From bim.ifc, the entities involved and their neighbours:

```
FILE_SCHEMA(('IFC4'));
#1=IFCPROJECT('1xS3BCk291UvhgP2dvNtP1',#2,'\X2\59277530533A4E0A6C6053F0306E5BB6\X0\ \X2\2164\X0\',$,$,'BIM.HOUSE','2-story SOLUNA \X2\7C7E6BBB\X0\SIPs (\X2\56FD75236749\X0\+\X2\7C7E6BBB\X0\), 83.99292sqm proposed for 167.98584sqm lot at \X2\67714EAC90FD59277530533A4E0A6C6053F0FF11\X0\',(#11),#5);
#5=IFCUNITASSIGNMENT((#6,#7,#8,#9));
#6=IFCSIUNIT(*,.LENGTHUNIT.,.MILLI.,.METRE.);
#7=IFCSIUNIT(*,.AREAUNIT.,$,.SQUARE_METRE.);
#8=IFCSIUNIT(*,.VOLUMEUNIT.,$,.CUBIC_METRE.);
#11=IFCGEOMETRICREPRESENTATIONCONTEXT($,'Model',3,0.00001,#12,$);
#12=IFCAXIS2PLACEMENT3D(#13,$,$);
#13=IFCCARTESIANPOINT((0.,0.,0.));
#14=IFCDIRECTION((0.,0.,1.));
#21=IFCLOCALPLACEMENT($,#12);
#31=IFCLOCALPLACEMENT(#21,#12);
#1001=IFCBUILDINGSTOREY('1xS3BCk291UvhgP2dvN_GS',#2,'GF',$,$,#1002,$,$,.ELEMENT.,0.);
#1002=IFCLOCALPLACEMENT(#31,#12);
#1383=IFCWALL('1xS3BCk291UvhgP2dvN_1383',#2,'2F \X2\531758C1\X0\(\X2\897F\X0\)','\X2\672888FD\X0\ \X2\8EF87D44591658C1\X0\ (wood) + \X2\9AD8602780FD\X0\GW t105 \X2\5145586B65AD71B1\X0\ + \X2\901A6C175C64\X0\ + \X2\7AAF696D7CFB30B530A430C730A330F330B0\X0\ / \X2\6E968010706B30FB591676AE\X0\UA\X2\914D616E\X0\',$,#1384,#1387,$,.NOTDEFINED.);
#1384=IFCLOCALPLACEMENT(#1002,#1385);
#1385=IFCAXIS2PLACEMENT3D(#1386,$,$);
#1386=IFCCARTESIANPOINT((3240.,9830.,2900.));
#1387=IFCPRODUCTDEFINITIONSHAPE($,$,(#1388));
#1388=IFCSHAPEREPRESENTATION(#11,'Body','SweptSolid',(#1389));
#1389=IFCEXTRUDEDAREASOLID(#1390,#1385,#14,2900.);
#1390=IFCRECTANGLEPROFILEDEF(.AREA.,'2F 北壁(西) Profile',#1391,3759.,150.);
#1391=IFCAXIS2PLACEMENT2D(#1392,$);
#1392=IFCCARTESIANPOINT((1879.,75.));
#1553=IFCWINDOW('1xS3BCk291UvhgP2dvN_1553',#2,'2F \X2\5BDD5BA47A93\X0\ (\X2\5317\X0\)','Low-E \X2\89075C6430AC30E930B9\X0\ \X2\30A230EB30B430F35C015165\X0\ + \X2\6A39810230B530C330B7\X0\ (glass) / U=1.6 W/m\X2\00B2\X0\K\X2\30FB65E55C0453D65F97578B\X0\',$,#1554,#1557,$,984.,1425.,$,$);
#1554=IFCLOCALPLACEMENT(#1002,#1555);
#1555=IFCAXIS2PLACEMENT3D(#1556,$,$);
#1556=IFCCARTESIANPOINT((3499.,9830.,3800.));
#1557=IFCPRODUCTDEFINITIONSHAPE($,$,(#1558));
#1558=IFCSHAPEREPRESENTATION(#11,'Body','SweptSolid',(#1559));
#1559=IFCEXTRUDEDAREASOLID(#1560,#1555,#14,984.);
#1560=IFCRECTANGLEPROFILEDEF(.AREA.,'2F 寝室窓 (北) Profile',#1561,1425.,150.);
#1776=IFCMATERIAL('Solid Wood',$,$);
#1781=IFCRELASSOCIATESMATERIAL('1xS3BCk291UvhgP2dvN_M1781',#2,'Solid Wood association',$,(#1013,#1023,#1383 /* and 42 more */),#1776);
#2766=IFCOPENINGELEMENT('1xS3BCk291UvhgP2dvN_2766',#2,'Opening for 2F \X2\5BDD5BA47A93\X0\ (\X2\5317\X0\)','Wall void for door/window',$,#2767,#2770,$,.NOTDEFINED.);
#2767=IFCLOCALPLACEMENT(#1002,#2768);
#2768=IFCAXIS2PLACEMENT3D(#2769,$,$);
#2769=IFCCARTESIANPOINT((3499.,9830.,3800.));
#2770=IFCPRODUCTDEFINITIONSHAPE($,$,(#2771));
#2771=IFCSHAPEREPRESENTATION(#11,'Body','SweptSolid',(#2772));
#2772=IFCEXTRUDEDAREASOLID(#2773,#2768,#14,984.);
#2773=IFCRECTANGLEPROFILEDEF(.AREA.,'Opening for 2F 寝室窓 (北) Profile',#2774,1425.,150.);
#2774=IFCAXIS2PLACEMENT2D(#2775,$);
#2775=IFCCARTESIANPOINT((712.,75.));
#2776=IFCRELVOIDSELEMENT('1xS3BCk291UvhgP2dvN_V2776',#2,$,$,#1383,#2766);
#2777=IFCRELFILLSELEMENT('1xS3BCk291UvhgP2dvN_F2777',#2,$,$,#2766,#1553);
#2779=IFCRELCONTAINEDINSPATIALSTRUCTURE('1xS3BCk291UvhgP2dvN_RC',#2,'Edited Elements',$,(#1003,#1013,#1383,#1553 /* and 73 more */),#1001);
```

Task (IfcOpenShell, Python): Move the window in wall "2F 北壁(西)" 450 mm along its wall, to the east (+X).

```python
import ifcopenshell
import ifcopenshell.api.geometry
import ifcopenshell.util.placement
import ifcopenshell.util.unit

model = ifcopenshell.open("bim.ifc")
unit_scale = ifcopenshell.util.unit.calculate_unit_scale(model)

window = model.by_guid("1xS3BCk291UvhgP2dvN_1553")
opening = window.FillsVoids[0].RelatingOpeningElement
wall = opening.VoidsElements[0].RelatingBuildingElement

wall_matrix = ifcopenshell.util.placement.get_local_placement(wall.ObjectPlacement)
shift = wall_matrix[:3, 0] * 0.45 / unit_scale
before = ifcopenshell.util.placement.get_local_placement(window.ObjectPlacement)[:3, 3].copy()

# The window is not placed relative to its opening, so move both.
for product in (opening, window):
    matrix = ifcopenshell.util.placement.get_local_placement(product.ObjectPlacement)
    matrix[:3, 3] += shift
    ifcopenshell.api.geometry.edit_object_placement(model, product=product, matrix=matrix, is_si=False)

after = ifcopenshell.util.placement.get_local_placement(window.ObjectPlacement)[:3, 3]
print("window moved by", (after - before).round(3) + 0.0)

model.write("bim-out.ifc")
```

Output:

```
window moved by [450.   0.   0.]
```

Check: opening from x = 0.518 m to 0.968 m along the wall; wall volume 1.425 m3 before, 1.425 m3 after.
